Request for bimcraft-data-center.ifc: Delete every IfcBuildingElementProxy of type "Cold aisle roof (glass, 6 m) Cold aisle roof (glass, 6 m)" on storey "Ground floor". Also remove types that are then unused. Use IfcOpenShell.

First a look at what the model holds.

```python
import ifcopenshell
import ifcopenshell.util.element

model = ifcopenshell.open("bimcraft-data-center.ifc")
print(model.schema)
storey = next(s for s in model.by_type("IfcBuildingStorey") if s.Name == "Ground floor")
proxies = [e for e in ifcopenshell.util.element.get_decomposition(storey) if e.is_a("IfcBuildingElementProxy")]
seen = {}
for e in proxies:
    element_type = ifcopenshell.util.element.get_type(e)
    name = element_type.Name if element_type not in (None, e) else None
    seen[name] = seen.get(name, 0) + 1
for name, count in sorted(seen.items(), key=str):
    print(count, "x", name)
```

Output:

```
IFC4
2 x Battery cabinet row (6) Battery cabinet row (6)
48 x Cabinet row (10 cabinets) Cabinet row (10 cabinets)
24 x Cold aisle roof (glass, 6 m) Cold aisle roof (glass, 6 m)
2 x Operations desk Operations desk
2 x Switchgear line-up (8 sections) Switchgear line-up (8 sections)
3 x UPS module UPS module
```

```python
import ifcopenshell
import ifcopenshell.api.root
import ifcopenshell.util.element

model = ifcopenshell.open("bimcraft-data-center.ifc")

storey = next(s for s in model.by_type("IfcBuildingStorey") if s.Name == "Ground floor")
proxies = [e for e in ifcopenshell.util.element.get_decomposition(storey) if e.is_a("IfcBuildingElementProxy")]
targets = [e for e in proxies if (t := ifcopenshell.util.element.get_type(e)) not in (None, e) and t.Name == "Cold aisle roof (glass, 6 m) Cold aisle roof (glass, 6 m)"]
types = {ifcopenshell.util.element.get_type(e) for e in targets} - {None, *targets}

for e in targets:
    ifcopenshell.api.root.remove_product(model, product=e)
print(len(targets), "removed")

unused = [t for t in types if not ifcopenshell.util.element.get_types(t)]
for t in unused:
    ifcopenshell.api.root.remove_product(model, product=t)
print(len(unused), "unused types removed")

model.write("bimcraft-data-center-out.ifc")
```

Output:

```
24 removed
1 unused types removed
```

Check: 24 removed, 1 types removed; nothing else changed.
